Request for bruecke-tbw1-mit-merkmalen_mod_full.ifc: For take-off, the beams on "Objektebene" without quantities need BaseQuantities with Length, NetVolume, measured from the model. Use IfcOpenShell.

First a look at what the model holds.

```python
import ifcopenshell
import ifcopenshell.util.element
import ifcopenshell.util.unit

model = ifcopenshell.open("bruecke-tbw1-mit-merkmalen_mod_full.ifc")
print(model.schema)
for unit_type in ("LENGTHUNIT", "AREAUNIT", "VOLUMEUNIT"):
    print(unit_type, ifcopenshell.util.unit.calculate_unit_scale(model, unit_type))
storey = next(s for s in model.by_type("IfcBuildingStorey") if s.Name == "Objektebene")
beams = [e for e in ifcopenshell.util.element.get_decomposition(storey) if e.is_a("IfcBeam")]
for e in sorted(beams, key=lambda e: e.id()):
    print(e.id(), e.is_a(), e.Name, list(ifcopenshell.util.element.get_psets(e, qtos_only=True)), sep=" | ")
```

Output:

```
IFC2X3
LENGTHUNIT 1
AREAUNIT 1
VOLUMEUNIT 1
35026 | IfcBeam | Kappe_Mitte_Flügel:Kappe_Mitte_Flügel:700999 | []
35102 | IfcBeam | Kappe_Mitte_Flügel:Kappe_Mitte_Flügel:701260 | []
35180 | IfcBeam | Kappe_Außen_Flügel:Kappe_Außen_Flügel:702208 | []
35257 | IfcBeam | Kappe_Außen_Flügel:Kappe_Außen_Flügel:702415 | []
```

```python
import ifcopenshell
import ifcopenshell.api.pset
import ifcopenshell.geom
import ifcopenshell.util.element
import ifcopenshell.util.shape
import ifcopenshell.util.unit

model = ifcopenshell.open("bruecke-tbw1-mit-merkmalen_mod_full.ifc")
unit_scale = ifcopenshell.util.unit.calculate_unit_scale(model)
volume_scale = ifcopenshell.util.unit.calculate_unit_scale(model, "VOLUMEUNIT")
settings = ifcopenshell.geom.settings()

storey = next(s for s in model.by_type("IfcBuildingStorey") if s.Name == "Objektebene")
beams = [e for e in ifcopenshell.util.element.get_decomposition(storey) if e.is_a("IfcBeam")]

for e in sorted(beams, key=lambda e: e.id()):
    if ifcopenshell.util.element.get_psets(e, qtos_only=True, should_inherit=False):
        continue
    # Geometry comes back in metres, in the element's own axes.
    shape = ifcopenshell.geom.create_shape(settings, e)
    values = {
        "Length": ifcopenshell.util.shape.get_max_xyz(shape.geometry) / unit_scale,
        "NetVolume": ifcopenshell.util.shape.get_volume(shape.geometry) / volume_scale,
    }
    qto = ifcopenshell.api.pset.add_qto(model, product=e, name="BaseQuantities")
    ifcopenshell.api.pset.edit_qto(model, qto=qto, properties=values)
    print(e.id(), {k: round(v, 3) for k, v in values.items()})

model.write("bruecke-tbw1-mit-merkmalen_mod_full_v2.ifc")
```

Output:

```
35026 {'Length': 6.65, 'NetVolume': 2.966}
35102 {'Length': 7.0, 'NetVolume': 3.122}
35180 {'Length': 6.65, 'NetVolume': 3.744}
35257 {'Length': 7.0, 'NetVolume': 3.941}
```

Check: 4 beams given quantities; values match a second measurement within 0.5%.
